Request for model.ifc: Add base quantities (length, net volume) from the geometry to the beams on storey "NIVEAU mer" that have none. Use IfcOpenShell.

First a look at what the model holds.

```python
import ifcopenshell
import ifcopenshell.util.element
import ifcopenshell.util.unit

model = ifcopenshell.open("model.ifc")
print(model.schema)
for unit_type in ("LENGTHUNIT", "AREAUNIT", "VOLUMEUNIT"):
    print(unit_type, ifcopenshell.util.unit.calculate_unit_scale(model, unit_type))
storey = next(s for s in model.by_type("IfcBuildingStorey") if s.Name == "NIVEAU mer")
beams = [e for e in ifcopenshell.util.element.get_decomposition(storey) if e.is_a("IfcBeam")]
for e in sorted(beams, key=lambda e: e.id()):
    print(e.id(), e.is_a(), e.Name, list(ifcopenshell.util.element.get_psets(e, qtos_only=True)), sep=" | ")
```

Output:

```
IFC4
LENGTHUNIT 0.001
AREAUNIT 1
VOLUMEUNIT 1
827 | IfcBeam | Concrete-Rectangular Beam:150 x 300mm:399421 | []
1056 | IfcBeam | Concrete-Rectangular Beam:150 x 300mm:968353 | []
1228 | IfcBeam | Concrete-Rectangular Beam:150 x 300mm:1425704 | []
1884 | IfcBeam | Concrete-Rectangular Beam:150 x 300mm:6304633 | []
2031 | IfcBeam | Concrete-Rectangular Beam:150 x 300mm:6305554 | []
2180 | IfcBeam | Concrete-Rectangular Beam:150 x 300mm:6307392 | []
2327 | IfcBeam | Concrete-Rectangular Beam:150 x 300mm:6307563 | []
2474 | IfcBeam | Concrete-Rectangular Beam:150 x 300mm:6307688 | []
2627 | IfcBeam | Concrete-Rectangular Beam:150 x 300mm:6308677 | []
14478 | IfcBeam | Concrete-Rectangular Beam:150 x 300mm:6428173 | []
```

```python
import ifcopenshell
import ifcopenshell.api.pset
import ifcopenshell.geom
import ifcopenshell.util.element
import ifcopenshell.util.shape
import ifcopenshell.util.unit

model = ifcopenshell.open("model.ifc")
unit_scale = ifcopenshell.util.unit.calculate_unit_scale(model)
volume_scale = ifcopenshell.util.unit.calculate_unit_scale(model, "VOLUMEUNIT")
settings = ifcopenshell.geom.settings()

storey = next(s for s in model.by_type("IfcBuildingStorey") if s.Name == "NIVEAU mer")
beams = [e for e in ifcopenshell.util.element.get_decomposition(storey) if e.is_a("IfcBeam")]

for e in sorted(beams, key=lambda e: e.id()):
    if ifcopenshell.util.element.get_psets(e, qtos_only=True, should_inherit=False):
        continue
    # Geometry comes back in metres, in the element's own axes.
    shape = ifcopenshell.geom.create_shape(settings, e)
    values = {
        "Length": ifcopenshell.util.shape.get_max_xyz(shape.geometry) / unit_scale,
        "NetVolume": ifcopenshell.util.shape.get_volume(shape.geometry) / volume_scale,
    }
    qto = ifcopenshell.api.pset.add_qto(model, product=e, name="Qto_BeamBaseQuantities")
    ifcopenshell.api.pset.edit_qto(model, qto=qto, properties=values)
    print(e.id(), {k: round(v, 3) for k, v in values.items()})

model.write("model_v2.ifc")
```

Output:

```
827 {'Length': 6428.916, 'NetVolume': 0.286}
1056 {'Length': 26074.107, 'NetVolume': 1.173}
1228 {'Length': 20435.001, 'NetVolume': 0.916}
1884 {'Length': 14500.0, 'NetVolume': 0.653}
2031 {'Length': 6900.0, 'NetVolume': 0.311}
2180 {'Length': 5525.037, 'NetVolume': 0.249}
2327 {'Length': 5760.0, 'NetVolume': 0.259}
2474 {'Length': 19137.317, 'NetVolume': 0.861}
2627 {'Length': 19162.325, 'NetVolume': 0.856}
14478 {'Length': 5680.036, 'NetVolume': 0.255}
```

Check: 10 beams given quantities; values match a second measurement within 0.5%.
